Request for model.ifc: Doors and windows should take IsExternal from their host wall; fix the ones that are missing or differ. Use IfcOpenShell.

First a look at what the model holds.

```python
import ifcopenshell
import ifcopenshell.util.element

model = ifcopenshell.open("model.ifc")
print(model.schema)
seen = {}
for e in model.by_type("IfcDoor") + model.by_type("IfcWindow"):
    if not e.FillsVoids:
        continue
    host = e.FillsVoids[0].RelatingOpeningElement.VoidsElements[0].RelatingBuildingElement
    own = ifcopenshell.util.element.get_pset(e, f"Pset_{e.is_a()[3:].removesuffix('StandardCase')}Common", "IsExternal")
    wall = ifcopenshell.util.element.get_pset(host, "Pset_WallCommon", "IsExternal")
    seen[e.is_a(), own, wall] = seen.get((e.is_a(), own, wall), 0) + 1
for (cls, own, wall), count in sorted(seen.items(), key=str):
    print(count, cls, "IsExternal:", own, "| host wall:", wall)
```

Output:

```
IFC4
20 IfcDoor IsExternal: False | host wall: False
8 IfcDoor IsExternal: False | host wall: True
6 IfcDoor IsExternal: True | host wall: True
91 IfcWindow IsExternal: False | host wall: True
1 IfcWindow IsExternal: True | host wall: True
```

```python
import ifcopenshell
import ifcopenshell.api.pset
import ifcopenshell.util.element

model = ifcopenshell.open("model.ifc")

count = 0
for ifc_class, pset_name in (("IfcDoor", "Pset_DoorCommon"), ("IfcWindow", "Pset_WindowCommon")):
    for e in model.by_type(ifc_class):
        if not e.FillsVoids:
            continue
        host = e.FillsVoids[0].RelatingOpeningElement.VoidsElements[0].RelatingBuildingElement
        external = ifcopenshell.util.element.get_pset(host, "Pset_WallCommon", "IsExternal")
        if external is None or ifcopenshell.util.element.get_pset(e, pset_name, "IsExternal") == external:
            continue
        pset = ifcopenshell.api.pset.add_pset(model, product=e, name=pset_name)
        ifcopenshell.api.pset.edit_pset(model, pset=pset, properties={"IsExternal": external})
        count += 1

print(count, "updated")

model.write("model_v2.ifc")
```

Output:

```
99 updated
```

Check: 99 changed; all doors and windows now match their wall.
